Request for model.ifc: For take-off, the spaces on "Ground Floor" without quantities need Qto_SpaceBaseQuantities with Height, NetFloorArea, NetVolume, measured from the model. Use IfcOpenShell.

First a look at what the model holds.

```python
import ifcopenshell
import ifcopenshell.util.element
import ifcopenshell.util.unit

model = ifcopenshell.open("model.ifc")
print(model.schema)
for unit_type in ("LENGTHUNIT", "AREAUNIT", "VOLUMEUNIT"):
    print(unit_type, ifcopenshell.util.unit.calculate_unit_scale(model, unit_type))
storey = next(s for s in model.by_type("IfcBuildingStorey") if s.Name == "Ground Floor")
spaces = [e for e in ifcopenshell.util.element.get_decomposition(storey) if e.is_a("IfcSpace")]
for e in sorted(spaces, key=lambda e: e.id()):
    print(e.id(), e.is_a(), e.Name, list(ifcopenshell.util.element.get_psets(e, qtos_only=True)), sep=" | ")
```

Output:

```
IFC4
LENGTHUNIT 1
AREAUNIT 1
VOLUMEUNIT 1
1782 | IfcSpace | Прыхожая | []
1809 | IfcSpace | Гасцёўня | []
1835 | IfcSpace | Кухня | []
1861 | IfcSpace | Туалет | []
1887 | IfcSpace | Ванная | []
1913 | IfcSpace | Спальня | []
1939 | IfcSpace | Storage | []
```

```python
import ifcopenshell
import ifcopenshell.api.pset
import ifcopenshell.geom
import ifcopenshell.util.element
import ifcopenshell.util.shape
import ifcopenshell.util.unit

model = ifcopenshell.open("model.ifc")
unit_scale = ifcopenshell.util.unit.calculate_unit_scale(model)
area_scale = ifcopenshell.util.unit.calculate_unit_scale(model, "AREAUNIT")
volume_scale = ifcopenshell.util.unit.calculate_unit_scale(model, "VOLUMEUNIT")
settings = ifcopenshell.geom.settings()

storey = next(s for s in model.by_type("IfcBuildingStorey") if s.Name == "Ground Floor")
spaces = [e for e in ifcopenshell.util.element.get_decomposition(storey) if e.is_a("IfcSpace")]

for e in sorted(spaces, key=lambda e: e.id()):
    if ifcopenshell.util.element.get_psets(e, qtos_only=True, should_inherit=False):
        continue
    # Geometry comes back in metres, in the element's own axes.
    shape = ifcopenshell.geom.create_shape(settings, e)
    values = {
        "Height": ifcopenshell.util.shape.get_z(shape.geometry) / unit_scale,
        "NetFloorArea": ifcopenshell.util.shape.get_footprint_area(shape.geometry) / area_scale,
        "NetVolume": ifcopenshell.util.shape.get_volume(shape.geometry) / volume_scale,
    }
    qto = ifcopenshell.api.pset.add_qto(model, product=e, name="Qto_SpaceBaseQuantities")
    ifcopenshell.api.pset.edit_qto(model, qto=qto, properties=values)
    print(e.id(), {k: round(v, 3) for k, v in values.items()})

model.write("model_v2.ifc")
```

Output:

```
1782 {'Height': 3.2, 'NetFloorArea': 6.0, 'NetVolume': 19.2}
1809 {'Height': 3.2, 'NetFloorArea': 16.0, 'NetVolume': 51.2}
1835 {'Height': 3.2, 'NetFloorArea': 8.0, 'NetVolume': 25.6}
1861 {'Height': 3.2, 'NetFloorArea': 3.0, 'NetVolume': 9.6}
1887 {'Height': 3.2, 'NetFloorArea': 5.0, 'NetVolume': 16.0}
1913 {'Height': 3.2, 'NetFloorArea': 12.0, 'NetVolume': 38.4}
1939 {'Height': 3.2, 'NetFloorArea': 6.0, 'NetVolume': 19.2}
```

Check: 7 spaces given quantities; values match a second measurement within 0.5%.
